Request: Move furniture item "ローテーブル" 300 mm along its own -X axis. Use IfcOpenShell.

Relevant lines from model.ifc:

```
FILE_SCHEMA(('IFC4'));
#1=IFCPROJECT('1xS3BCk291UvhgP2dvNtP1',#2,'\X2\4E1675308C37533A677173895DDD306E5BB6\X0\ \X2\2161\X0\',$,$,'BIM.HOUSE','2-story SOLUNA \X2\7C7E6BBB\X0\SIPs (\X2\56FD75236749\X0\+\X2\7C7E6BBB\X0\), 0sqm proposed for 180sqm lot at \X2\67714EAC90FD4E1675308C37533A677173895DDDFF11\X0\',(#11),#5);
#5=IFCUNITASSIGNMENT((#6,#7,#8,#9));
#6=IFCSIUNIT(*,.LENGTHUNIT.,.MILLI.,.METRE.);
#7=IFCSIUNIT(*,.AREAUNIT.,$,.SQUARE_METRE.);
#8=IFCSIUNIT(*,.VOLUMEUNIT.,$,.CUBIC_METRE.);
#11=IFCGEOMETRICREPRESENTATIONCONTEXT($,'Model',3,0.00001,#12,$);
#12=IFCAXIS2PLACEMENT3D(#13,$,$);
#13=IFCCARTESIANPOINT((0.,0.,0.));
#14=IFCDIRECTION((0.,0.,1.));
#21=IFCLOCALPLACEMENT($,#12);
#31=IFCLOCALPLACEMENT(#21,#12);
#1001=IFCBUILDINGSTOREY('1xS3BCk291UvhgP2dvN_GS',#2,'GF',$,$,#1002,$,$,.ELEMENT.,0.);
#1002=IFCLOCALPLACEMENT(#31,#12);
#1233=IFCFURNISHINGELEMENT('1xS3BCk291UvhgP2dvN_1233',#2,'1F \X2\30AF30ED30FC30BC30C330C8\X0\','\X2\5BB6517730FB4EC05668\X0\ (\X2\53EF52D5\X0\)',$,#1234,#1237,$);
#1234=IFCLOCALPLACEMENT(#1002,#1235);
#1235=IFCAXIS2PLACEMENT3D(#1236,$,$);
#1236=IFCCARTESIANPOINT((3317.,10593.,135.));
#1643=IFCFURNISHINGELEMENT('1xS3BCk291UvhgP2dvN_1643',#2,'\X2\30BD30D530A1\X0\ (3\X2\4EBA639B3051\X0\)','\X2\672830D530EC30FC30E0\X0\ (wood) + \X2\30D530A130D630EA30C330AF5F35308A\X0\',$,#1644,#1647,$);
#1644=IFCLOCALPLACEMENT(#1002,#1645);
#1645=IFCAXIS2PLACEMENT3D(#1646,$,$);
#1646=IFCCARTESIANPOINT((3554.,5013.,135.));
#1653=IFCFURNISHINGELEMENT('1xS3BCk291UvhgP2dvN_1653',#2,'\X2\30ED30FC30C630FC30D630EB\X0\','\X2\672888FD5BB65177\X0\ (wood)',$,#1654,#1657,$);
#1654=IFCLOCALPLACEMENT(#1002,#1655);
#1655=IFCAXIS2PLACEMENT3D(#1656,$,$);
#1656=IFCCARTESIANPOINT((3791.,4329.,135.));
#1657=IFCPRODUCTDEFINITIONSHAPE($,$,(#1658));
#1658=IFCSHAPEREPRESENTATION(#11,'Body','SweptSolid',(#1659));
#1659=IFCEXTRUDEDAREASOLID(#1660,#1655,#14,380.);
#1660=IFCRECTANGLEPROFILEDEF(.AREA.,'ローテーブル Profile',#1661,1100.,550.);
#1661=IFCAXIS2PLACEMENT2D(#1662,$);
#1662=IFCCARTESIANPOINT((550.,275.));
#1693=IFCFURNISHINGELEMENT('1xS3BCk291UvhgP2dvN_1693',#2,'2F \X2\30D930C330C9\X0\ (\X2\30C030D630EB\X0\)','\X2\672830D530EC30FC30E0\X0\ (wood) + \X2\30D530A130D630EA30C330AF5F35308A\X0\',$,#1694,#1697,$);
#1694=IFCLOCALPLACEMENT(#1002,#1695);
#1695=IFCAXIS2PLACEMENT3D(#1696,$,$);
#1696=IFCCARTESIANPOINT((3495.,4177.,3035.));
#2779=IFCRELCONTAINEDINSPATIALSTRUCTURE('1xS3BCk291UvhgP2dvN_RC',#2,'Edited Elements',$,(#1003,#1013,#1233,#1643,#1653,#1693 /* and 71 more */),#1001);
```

```python
import ifcopenshell
import ifcopenshell.api.geometry
import ifcopenshell.util.placement

model = ifcopenshell.open("model.ifc")

item = model.by_id(1653)
matrix = ifcopenshell.util.placement.get_local_placement(item.ObjectPlacement)
matrix[:3, 3] -= matrix[:3, 0] * 300.0
ifcopenshell.api.geometry.edit_object_placement(model, product=item, matrix=matrix, is_si=False)

print(ifcopenshell.util.placement.get_local_placement(item.ObjectPlacement).round(3) + 0.0)

model.write("model_v2.ifc")
```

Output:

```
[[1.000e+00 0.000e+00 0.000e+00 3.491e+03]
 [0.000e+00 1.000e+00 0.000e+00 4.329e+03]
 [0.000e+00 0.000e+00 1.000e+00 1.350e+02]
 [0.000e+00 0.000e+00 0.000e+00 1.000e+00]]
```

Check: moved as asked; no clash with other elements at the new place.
